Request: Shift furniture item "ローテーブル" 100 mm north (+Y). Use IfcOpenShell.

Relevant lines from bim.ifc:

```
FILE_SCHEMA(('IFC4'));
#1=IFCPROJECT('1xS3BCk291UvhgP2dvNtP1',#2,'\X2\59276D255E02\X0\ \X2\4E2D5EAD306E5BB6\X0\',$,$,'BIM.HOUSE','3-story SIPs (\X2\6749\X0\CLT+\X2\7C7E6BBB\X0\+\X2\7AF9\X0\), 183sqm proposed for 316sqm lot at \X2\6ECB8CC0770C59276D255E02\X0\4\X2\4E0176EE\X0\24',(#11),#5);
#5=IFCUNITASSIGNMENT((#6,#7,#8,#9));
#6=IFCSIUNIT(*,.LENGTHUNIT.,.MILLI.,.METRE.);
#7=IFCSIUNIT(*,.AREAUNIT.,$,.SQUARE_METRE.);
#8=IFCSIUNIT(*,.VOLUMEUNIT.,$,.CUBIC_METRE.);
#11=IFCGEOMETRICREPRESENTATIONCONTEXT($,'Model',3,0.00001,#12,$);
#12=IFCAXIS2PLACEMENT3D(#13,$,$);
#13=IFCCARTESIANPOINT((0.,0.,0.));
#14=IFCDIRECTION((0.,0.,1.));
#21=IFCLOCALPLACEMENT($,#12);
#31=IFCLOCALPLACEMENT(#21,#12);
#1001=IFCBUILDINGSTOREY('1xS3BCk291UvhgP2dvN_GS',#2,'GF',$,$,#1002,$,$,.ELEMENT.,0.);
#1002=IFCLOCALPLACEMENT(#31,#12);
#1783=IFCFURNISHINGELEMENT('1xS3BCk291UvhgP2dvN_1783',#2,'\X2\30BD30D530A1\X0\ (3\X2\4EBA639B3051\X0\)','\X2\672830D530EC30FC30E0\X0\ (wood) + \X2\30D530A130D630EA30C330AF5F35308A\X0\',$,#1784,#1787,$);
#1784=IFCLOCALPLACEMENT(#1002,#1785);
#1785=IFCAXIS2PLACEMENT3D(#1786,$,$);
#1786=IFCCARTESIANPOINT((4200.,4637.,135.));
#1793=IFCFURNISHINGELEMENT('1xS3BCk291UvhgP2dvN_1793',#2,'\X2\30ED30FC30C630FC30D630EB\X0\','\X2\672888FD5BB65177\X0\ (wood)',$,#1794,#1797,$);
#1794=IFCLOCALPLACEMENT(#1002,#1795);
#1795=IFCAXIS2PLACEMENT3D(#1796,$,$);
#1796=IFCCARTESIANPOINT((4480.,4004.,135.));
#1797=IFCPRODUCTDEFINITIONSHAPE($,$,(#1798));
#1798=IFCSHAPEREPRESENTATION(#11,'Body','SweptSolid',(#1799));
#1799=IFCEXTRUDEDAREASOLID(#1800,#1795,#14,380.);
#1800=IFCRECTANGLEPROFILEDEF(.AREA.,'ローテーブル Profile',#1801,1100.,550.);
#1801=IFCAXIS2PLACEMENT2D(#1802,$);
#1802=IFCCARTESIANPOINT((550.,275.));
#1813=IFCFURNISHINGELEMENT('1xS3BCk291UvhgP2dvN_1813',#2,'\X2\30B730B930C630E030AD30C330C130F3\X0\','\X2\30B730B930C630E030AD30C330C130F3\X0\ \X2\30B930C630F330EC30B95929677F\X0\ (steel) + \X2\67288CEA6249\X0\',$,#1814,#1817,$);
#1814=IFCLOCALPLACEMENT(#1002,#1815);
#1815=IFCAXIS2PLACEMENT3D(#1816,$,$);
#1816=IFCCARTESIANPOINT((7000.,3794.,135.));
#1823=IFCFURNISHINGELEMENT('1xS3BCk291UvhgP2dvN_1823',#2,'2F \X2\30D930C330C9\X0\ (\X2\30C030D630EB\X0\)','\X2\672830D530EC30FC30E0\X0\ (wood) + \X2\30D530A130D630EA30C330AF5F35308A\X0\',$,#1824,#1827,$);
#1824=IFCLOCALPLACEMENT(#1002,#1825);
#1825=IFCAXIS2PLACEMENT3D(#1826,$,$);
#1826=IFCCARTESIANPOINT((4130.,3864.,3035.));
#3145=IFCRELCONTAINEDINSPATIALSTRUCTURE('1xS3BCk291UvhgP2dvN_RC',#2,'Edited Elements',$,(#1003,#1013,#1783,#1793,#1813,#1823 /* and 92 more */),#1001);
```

```python
import ifcopenshell
import ifcopenshell.api.geometry
import ifcopenshell.util.placement
import ifcopenshell.util.unit

model = ifcopenshell.open("bim.ifc")
unit_scale = ifcopenshell.util.unit.calculate_unit_scale(model)

item = model.by_guid("1xS3BCk291UvhgP2dvN_1793")
matrix = ifcopenshell.util.placement.get_local_placement(item.ObjectPlacement)
matrix[1, 3] += 0.1 / unit_scale
ifcopenshell.api.geometry.edit_object_placement(model, product=item, matrix=matrix, is_si=False)

print(ifcopenshell.util.placement.get_local_placement(item.ObjectPlacement).round(3) + 0.0)

model.write("bim_updated.ifc")
```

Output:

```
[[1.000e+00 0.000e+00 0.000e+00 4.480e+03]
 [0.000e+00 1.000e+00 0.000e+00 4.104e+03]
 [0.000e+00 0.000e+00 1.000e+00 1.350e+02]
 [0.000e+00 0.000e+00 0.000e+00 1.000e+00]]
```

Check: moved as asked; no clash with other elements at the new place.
